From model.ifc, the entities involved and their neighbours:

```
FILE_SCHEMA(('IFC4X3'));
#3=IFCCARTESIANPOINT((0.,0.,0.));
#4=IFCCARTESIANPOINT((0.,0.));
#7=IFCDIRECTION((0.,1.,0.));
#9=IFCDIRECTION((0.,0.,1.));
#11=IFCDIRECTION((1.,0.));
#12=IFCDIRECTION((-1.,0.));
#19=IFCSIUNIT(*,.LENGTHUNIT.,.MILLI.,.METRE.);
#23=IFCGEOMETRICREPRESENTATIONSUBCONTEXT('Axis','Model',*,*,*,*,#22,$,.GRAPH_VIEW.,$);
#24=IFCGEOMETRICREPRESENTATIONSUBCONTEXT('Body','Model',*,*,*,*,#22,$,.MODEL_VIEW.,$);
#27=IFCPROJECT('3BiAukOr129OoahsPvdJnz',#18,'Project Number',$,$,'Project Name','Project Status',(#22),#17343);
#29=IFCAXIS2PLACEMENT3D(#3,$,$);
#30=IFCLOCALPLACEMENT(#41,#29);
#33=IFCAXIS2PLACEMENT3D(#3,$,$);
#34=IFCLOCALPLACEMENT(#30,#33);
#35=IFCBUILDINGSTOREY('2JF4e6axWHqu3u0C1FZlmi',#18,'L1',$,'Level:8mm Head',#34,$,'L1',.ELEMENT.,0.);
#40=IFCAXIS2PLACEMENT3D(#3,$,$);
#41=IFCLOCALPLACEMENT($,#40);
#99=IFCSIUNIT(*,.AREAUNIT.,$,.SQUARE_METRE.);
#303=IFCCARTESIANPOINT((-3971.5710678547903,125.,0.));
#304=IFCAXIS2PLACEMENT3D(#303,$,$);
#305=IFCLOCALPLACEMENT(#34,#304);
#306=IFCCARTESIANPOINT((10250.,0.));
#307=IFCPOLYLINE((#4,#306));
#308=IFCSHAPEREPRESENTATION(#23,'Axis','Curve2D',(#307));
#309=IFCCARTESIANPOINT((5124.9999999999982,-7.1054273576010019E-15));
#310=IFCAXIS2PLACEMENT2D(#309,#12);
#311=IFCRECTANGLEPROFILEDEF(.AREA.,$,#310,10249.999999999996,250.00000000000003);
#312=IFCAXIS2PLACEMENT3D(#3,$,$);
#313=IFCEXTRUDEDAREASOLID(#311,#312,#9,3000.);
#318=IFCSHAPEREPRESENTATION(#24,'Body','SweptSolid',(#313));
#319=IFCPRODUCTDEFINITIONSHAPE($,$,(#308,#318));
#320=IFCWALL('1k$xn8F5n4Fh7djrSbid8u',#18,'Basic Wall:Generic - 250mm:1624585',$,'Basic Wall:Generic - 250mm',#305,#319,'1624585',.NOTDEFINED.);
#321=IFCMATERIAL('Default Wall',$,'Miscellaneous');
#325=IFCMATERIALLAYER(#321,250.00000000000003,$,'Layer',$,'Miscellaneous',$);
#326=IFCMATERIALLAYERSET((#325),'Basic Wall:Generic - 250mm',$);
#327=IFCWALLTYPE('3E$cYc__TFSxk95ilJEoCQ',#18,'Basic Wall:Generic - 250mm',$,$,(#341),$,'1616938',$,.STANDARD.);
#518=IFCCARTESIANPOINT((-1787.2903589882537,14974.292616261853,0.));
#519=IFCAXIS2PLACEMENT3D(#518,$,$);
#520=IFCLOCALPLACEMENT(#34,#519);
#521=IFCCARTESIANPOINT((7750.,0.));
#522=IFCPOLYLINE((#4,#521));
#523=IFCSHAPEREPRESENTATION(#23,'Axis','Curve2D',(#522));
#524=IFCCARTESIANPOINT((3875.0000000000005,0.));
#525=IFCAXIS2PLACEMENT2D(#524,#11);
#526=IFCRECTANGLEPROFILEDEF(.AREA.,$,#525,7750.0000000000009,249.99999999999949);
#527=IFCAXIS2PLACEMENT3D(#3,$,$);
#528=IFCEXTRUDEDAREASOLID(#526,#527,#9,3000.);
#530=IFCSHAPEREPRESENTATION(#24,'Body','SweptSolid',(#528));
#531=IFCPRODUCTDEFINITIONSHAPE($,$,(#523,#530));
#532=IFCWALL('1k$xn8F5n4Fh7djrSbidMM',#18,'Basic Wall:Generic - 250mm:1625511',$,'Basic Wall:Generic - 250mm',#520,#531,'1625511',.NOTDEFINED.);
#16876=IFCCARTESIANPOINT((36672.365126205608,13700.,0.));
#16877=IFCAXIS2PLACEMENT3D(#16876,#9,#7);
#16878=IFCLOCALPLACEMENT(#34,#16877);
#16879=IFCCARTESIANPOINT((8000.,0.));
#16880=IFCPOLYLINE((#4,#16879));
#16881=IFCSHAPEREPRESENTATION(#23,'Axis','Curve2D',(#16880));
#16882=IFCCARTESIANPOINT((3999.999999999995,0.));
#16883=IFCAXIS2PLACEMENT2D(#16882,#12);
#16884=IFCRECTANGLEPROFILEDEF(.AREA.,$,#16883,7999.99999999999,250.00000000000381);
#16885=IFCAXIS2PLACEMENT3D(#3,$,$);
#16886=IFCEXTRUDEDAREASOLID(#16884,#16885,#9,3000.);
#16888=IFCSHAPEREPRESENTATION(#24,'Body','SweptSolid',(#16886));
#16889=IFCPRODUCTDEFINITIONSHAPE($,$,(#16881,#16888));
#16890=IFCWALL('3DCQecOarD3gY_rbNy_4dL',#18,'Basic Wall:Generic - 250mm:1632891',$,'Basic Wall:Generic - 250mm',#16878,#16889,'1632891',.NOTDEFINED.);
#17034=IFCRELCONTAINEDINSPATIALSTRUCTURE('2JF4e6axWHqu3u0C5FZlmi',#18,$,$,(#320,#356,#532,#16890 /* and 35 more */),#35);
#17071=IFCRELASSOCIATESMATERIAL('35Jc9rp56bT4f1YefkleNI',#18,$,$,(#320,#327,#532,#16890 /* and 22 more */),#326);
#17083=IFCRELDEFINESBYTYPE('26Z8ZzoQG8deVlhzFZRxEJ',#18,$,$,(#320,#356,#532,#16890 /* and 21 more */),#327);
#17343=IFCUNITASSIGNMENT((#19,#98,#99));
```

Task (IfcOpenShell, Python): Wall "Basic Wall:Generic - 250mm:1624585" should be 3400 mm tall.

```python
import ifcopenshell
import ifcopenshell.geom
import ifcopenshell.util.representation
import ifcopenshell.util.shape
import ifcopenshell.util.unit

model = ifcopenshell.open("model.ifc")
unit_scale = ifcopenshell.util.unit.calculate_unit_scale(model)
settings = ifcopenshell.geom.settings()


def volume(element):
    """Net volume in cubic metres, openings subtracted."""
    shape = ifcopenshell.geom.create_shape(settings, element)
    return ifcopenshell.util.shape.get_volume(shape.geometry)


wall = model.by_guid("1k$xn8F5n4Fh7djrSbid8u")
before = volume(wall)

body = ifcopenshell.util.representation.get_representation(wall, "Model", "Body")
solid = body.Items[0]
old_height = solid.Depth
solid.Depth = 3.4 / unit_scale
after = volume(wall)

print(f"height {old_height:g} -> {solid.Depth:g}, volume {before:.3f} -> {after:.3f} m3")

model.write("model_edited.ifc")
```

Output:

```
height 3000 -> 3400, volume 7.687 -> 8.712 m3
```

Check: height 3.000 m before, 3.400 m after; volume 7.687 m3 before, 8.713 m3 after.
